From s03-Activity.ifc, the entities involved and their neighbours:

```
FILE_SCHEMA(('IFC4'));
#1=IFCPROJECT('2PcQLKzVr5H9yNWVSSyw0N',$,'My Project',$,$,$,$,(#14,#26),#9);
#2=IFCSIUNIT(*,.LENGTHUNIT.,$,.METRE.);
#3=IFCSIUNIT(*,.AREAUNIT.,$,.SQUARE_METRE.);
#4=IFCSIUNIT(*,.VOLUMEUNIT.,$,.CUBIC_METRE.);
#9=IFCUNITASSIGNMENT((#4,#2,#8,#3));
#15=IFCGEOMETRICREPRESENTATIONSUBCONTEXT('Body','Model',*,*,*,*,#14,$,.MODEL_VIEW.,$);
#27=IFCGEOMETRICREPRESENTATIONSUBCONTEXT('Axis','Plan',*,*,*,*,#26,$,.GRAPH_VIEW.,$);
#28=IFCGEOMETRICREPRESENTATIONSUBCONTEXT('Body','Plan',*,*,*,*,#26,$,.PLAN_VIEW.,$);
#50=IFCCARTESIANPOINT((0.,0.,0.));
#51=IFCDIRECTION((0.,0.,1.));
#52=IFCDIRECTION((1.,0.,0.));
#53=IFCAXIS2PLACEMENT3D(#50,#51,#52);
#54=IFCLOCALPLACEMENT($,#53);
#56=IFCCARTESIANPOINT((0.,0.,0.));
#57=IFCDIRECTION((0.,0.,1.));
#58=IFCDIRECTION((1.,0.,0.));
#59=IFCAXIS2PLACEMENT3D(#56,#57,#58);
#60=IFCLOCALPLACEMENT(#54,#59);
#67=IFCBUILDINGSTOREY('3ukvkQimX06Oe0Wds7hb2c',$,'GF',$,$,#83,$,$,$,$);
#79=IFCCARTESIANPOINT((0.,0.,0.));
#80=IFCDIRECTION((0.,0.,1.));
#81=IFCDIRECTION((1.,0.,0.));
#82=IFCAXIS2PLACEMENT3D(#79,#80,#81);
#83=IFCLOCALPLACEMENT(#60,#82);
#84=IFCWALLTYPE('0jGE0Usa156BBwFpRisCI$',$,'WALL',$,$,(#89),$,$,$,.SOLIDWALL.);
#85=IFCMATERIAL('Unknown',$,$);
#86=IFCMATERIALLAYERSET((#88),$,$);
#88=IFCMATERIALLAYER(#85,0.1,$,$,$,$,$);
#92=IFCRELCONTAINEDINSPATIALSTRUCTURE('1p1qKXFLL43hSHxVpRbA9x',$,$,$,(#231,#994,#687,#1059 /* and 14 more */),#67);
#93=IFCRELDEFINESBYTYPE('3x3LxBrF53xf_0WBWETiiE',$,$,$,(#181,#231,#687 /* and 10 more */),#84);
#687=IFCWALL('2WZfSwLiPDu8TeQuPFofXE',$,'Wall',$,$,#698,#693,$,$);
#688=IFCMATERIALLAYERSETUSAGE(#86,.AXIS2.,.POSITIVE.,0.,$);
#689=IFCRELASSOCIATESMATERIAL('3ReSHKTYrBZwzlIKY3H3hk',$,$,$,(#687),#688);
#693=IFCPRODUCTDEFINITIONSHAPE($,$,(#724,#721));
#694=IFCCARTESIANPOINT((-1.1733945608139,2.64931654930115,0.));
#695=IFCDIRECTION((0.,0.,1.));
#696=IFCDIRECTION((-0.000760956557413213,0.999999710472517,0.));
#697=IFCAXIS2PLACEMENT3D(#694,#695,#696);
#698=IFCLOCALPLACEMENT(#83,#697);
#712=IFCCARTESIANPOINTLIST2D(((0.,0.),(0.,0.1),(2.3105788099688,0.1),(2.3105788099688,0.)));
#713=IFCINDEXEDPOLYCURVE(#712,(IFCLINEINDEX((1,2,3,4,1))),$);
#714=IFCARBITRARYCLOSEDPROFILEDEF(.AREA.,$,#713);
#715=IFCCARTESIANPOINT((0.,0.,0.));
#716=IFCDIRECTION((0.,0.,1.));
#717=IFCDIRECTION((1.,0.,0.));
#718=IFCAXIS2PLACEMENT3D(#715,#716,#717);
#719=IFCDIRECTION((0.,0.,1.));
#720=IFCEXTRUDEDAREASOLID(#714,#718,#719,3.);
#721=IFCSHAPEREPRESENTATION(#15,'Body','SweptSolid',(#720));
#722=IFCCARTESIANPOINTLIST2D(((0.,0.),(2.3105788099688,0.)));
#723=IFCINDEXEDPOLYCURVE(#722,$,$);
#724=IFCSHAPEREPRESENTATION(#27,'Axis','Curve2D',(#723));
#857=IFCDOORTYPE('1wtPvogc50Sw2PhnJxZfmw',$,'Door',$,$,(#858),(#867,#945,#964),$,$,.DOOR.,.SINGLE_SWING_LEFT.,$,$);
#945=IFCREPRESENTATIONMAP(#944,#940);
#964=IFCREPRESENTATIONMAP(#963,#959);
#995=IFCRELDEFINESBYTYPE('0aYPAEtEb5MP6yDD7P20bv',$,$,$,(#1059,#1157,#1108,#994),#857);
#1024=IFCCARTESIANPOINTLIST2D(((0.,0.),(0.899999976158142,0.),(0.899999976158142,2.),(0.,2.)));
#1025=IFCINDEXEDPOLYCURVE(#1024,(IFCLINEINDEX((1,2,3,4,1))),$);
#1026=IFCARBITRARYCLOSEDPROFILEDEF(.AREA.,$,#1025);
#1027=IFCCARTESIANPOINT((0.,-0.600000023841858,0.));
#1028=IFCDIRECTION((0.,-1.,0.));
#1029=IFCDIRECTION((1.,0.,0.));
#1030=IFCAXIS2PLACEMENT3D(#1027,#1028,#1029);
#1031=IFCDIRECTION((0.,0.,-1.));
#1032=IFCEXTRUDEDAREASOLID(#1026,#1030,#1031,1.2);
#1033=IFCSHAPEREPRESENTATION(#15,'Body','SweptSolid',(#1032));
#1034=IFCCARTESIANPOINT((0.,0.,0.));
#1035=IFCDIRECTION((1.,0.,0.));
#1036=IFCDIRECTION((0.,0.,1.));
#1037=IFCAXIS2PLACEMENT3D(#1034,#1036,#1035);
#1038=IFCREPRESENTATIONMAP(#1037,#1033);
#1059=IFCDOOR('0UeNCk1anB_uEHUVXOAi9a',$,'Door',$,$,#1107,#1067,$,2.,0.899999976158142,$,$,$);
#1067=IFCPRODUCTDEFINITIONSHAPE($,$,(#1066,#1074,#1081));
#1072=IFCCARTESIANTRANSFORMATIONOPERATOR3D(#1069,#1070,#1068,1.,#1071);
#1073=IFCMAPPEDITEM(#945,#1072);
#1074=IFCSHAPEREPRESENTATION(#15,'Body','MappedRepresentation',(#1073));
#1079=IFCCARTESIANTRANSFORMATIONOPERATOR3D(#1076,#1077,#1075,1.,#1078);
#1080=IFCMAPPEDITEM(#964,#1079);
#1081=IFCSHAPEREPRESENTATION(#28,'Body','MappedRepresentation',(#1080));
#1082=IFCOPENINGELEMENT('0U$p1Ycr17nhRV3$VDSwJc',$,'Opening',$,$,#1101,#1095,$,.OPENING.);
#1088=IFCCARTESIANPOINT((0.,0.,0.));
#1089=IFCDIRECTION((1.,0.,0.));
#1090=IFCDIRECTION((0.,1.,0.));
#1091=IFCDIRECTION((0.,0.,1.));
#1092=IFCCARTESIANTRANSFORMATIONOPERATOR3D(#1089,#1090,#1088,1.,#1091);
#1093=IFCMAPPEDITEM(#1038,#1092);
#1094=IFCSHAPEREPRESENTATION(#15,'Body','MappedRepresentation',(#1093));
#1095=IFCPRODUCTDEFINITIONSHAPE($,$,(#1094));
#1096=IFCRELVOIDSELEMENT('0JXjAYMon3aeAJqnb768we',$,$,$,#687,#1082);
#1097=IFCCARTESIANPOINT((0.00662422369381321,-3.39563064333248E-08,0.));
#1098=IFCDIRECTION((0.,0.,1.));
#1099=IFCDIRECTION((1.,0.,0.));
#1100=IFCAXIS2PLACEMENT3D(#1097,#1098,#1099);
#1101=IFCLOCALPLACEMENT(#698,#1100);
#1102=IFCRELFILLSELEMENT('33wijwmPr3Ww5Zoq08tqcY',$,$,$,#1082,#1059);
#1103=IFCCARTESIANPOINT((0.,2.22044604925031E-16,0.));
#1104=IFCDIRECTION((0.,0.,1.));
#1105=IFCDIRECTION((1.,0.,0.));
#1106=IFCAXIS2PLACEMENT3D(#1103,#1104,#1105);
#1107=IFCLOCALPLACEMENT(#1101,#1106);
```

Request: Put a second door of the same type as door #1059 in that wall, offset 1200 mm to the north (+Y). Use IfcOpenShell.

```python
import ifcopenshell
import ifcopenshell.api.feature
import ifcopenshell.api.geometry
import ifcopenshell.api.root
import ifcopenshell.geom
import ifcopenshell.util.element
import ifcopenshell.util.placement
import ifcopenshell.util.shape
import ifcopenshell.util.unit

model = ifcopenshell.open("s03-Activity.ifc")
unit_scale = ifcopenshell.util.unit.calculate_unit_scale(model)
settings = ifcopenshell.geom.settings()


def volume(element):
    """Net volume in cubic metres, openings subtracted."""
    shape = ifcopenshell.geom.create_shape(settings, element)
    return ifcopenshell.util.shape.get_volume(shape.geometry)


door = model.by_id(1059)
opening = door.FillsVoids[0].RelatingOpeningElement
wall = opening.VoidsElements[0].RelatingBuildingElement
before = volume(wall)
shift = ifcopenshell.util.placement.get_local_placement(wall.ObjectPlacement)[:3, 0] * 1.2 / unit_scale

# copy_class copies the void relationship, type, container and properties, but no geometry.
new_opening = ifcopenshell.api.root.copy_class(model, product=opening)
new_opening.Representation = ifcopenshell.util.element.copy_deep(
    model, opening.Representation, exclude=["IfcGeometricRepresentationContext", "IfcRepresentationMap"]
)
new_door = ifcopenshell.api.root.copy_class(model, product=door)
new_door.Representation = ifcopenshell.util.element.copy_deep(
    model, door.Representation, exclude=["IfcGeometricRepresentationContext", "IfcRepresentationMap"]
)
ifcopenshell.api.feature.add_filling(model, opening=new_opening, element=new_door)

for old, new in ((opening, new_opening), (door, new_door)):
    matrix = ifcopenshell.util.placement.get_local_placement(old.ObjectPlacement)
    matrix[:3, 3] += shift
    ifcopenshell.api.geometry.edit_object_placement(model, product=new, matrix=matrix, is_si=False)

after = volume(wall)

print(f"wall volume {before:.3f} -> {after:.3f} m3")

model.write("s03-Activity-out.ifc")
```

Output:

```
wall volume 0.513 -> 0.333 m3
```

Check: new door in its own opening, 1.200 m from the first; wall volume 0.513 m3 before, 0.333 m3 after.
